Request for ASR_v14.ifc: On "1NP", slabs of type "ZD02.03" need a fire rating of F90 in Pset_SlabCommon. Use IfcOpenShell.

First a look at what the model holds.

```python
import ifcopenshell
import ifcopenshell.util.element

model = ifcopenshell.open("ASR_v14.ifc")
print(model.schema)
storey = next(s for s in model.by_type("IfcBuildingStorey") if s.Name == "1NP")
slabs = [e for e in ifcopenshell.util.element.get_decomposition(storey) if e.is_a("IfcSlab")]
seen = {}
for e in slabs:
    element_type = ifcopenshell.util.element.get_type(e)
    key = (element_type.Name if element_type != e and element_type else None, ifcopenshell.util.element.get_pset(e, "Pset_SlabCommon", "FireRating"))
    seen[key] = seen.get(key, 0) + 1
for (name, value), count in sorted(seen.items(), key=str):
    print(count, "x", name, "|", value)
```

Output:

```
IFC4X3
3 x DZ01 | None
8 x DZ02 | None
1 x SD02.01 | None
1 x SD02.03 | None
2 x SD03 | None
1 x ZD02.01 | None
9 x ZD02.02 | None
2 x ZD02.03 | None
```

```python
import ifcopenshell
import ifcopenshell.api.pset
import ifcopenshell.util.element

model = ifcopenshell.open("ASR_v14.ifc")

storey = next(s for s in model.by_type("IfcBuildingStorey") if s.Name == "1NP")
slabs = [e for e in ifcopenshell.util.element.get_decomposition(storey) if e.is_a("IfcSlab")]

count = 0
for e in slabs:
    element_type = ifcopenshell.util.element.get_type(e)
    if element_type in (None, e) or element_type.Name != "ZD02.03":
        continue
    # add_pset returns the element's existing set when there is one.
    pset = ifcopenshell.api.pset.add_pset(model, product=e, name="Pset_SlabCommon")
    ifcopenshell.api.pset.edit_pset(model, pset=pset, properties={"FireRating": "F90"})
    count += 1

print(count, "slabs updated")

model.write("ASR_v14_rev.ifc")
```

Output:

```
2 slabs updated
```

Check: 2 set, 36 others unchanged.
